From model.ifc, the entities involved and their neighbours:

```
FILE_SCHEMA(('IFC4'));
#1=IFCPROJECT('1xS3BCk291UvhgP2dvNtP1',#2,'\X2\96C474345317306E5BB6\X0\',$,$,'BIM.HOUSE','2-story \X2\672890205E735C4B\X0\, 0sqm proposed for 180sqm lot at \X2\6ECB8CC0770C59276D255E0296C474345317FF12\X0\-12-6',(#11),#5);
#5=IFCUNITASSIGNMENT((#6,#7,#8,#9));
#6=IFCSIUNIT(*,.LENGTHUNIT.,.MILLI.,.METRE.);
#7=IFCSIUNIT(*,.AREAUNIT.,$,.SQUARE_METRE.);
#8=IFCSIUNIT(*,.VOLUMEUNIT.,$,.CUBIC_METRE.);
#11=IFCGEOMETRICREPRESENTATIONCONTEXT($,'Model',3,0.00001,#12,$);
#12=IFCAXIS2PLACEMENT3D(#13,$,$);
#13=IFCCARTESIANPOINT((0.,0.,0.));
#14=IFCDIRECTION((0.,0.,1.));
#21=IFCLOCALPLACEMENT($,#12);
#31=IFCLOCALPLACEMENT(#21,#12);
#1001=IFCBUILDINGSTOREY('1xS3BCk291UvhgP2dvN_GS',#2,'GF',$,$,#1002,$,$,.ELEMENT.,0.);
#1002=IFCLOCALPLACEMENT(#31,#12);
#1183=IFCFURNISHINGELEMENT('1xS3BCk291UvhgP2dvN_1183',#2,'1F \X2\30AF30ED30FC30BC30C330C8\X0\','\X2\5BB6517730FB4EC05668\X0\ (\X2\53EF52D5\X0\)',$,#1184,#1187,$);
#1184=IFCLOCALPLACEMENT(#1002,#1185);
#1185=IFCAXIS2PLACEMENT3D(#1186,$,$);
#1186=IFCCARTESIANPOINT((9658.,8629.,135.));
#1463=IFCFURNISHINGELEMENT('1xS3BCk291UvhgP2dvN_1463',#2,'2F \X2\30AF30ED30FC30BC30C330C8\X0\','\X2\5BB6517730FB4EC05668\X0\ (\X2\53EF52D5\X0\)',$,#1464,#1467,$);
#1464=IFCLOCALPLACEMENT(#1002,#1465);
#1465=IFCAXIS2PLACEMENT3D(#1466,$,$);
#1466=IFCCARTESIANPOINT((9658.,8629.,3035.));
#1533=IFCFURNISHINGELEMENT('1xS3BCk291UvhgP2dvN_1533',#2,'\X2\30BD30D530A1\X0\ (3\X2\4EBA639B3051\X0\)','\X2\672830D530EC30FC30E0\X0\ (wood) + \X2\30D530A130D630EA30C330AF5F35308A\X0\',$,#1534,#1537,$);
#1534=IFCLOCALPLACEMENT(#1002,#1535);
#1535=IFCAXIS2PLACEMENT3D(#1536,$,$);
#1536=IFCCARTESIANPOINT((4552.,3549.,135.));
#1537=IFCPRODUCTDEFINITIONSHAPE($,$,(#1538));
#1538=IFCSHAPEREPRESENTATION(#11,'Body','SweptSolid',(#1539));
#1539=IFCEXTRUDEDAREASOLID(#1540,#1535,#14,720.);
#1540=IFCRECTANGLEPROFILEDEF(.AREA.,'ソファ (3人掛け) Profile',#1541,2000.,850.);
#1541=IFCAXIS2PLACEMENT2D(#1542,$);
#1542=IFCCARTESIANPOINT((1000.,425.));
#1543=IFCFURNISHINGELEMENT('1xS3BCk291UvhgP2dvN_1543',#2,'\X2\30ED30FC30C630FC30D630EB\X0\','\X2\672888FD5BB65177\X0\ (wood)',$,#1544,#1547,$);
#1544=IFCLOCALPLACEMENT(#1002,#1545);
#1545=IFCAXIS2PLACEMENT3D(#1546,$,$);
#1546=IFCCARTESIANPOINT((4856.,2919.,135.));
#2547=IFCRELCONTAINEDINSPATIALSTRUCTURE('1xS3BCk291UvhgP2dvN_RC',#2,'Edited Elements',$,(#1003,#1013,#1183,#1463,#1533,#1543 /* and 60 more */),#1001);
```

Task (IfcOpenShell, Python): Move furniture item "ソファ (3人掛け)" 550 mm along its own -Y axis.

```python
import ifcopenshell
import ifcopenshell.api.geometry
import ifcopenshell.util.placement
import ifcopenshell.util.unit

model = ifcopenshell.open("model.ifc")
unit_scale = ifcopenshell.util.unit.calculate_unit_scale(model)

item = model.by_guid("1xS3BCk291UvhgP2dvN_1533")
matrix = ifcopenshell.util.placement.get_local_placement(item.ObjectPlacement)
matrix[:3, 3] -= matrix[:3, 1] * 0.55 / unit_scale
ifcopenshell.api.geometry.edit_object_placement(model, product=item, matrix=matrix, is_si=False)

print(ifcopenshell.util.placement.get_local_placement(item.ObjectPlacement).round(3) + 0.0)

model.write("model_updated.ifc")
```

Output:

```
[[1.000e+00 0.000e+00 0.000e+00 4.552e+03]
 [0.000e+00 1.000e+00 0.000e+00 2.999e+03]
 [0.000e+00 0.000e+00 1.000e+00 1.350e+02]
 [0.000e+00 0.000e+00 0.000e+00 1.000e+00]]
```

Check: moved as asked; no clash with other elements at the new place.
